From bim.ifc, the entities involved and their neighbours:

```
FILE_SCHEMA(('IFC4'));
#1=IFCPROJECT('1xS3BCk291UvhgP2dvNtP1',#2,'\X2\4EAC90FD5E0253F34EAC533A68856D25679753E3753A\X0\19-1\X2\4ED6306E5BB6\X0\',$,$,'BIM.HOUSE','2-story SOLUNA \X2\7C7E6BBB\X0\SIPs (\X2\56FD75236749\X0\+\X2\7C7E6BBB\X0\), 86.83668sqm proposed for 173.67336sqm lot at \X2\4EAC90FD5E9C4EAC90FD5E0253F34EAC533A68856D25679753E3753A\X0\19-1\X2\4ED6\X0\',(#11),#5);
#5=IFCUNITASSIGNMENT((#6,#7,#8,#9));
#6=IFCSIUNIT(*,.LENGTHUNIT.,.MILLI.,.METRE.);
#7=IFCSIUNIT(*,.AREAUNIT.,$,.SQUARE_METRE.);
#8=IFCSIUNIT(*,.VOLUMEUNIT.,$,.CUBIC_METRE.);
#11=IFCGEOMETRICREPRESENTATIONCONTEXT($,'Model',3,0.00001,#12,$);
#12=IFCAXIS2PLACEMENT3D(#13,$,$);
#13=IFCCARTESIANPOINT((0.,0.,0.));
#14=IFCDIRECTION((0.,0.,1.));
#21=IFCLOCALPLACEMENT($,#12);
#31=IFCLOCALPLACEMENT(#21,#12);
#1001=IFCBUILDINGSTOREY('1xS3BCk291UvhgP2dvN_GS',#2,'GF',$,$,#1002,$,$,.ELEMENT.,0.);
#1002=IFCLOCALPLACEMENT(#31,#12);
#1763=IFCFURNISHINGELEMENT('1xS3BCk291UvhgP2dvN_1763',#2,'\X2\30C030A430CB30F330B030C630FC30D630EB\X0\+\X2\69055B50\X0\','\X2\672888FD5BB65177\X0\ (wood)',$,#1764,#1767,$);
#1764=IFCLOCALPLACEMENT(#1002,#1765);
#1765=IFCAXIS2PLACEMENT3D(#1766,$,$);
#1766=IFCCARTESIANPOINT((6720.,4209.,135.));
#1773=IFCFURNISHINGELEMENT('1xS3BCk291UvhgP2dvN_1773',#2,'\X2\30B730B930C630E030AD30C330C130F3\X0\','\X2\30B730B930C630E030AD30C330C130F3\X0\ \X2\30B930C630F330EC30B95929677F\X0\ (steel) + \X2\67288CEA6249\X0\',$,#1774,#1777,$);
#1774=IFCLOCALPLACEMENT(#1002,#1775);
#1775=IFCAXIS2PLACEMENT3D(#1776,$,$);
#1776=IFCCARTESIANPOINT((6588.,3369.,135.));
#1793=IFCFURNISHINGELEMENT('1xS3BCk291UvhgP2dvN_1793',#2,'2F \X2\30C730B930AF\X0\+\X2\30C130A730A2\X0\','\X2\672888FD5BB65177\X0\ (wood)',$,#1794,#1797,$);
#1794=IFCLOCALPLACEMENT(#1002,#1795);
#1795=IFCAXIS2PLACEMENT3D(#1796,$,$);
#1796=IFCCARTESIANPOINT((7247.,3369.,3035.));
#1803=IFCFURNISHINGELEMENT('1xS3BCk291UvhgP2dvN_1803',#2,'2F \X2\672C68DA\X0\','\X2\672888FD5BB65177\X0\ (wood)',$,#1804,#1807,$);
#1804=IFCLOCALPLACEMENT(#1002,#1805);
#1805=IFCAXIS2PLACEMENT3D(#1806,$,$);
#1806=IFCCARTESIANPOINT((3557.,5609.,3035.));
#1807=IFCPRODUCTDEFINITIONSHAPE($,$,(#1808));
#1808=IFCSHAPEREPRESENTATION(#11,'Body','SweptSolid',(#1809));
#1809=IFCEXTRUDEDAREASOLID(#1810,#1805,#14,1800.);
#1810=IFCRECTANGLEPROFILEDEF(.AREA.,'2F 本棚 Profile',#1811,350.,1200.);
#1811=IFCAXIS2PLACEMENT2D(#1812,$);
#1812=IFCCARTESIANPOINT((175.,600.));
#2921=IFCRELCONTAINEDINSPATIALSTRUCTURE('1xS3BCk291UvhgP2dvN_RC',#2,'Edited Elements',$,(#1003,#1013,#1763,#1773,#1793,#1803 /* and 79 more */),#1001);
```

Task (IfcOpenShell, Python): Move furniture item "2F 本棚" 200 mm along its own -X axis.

```python
import ifcopenshell
import ifcopenshell.api.geometry
import ifcopenshell.util.placement
import ifcopenshell.util.unit

model = ifcopenshell.open("bim.ifc")
unit_scale = ifcopenshell.util.unit.calculate_unit_scale(model)

item = model.by_guid("1xS3BCk291UvhgP2dvN_1803")
matrix = ifcopenshell.util.placement.get_local_placement(item.ObjectPlacement)
matrix[:3, 3] -= matrix[:3, 0] * 0.2 / unit_scale
ifcopenshell.api.geometry.edit_object_placement(model, product=item, matrix=matrix, is_si=False)

print(ifcopenshell.util.placement.get_local_placement(item.ObjectPlacement).round(3) + 0.0)

model.write("bim_updated.ifc")
```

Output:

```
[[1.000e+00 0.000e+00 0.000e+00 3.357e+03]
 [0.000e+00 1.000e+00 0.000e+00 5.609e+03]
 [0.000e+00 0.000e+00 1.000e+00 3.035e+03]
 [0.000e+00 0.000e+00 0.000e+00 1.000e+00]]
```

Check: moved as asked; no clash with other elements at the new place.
